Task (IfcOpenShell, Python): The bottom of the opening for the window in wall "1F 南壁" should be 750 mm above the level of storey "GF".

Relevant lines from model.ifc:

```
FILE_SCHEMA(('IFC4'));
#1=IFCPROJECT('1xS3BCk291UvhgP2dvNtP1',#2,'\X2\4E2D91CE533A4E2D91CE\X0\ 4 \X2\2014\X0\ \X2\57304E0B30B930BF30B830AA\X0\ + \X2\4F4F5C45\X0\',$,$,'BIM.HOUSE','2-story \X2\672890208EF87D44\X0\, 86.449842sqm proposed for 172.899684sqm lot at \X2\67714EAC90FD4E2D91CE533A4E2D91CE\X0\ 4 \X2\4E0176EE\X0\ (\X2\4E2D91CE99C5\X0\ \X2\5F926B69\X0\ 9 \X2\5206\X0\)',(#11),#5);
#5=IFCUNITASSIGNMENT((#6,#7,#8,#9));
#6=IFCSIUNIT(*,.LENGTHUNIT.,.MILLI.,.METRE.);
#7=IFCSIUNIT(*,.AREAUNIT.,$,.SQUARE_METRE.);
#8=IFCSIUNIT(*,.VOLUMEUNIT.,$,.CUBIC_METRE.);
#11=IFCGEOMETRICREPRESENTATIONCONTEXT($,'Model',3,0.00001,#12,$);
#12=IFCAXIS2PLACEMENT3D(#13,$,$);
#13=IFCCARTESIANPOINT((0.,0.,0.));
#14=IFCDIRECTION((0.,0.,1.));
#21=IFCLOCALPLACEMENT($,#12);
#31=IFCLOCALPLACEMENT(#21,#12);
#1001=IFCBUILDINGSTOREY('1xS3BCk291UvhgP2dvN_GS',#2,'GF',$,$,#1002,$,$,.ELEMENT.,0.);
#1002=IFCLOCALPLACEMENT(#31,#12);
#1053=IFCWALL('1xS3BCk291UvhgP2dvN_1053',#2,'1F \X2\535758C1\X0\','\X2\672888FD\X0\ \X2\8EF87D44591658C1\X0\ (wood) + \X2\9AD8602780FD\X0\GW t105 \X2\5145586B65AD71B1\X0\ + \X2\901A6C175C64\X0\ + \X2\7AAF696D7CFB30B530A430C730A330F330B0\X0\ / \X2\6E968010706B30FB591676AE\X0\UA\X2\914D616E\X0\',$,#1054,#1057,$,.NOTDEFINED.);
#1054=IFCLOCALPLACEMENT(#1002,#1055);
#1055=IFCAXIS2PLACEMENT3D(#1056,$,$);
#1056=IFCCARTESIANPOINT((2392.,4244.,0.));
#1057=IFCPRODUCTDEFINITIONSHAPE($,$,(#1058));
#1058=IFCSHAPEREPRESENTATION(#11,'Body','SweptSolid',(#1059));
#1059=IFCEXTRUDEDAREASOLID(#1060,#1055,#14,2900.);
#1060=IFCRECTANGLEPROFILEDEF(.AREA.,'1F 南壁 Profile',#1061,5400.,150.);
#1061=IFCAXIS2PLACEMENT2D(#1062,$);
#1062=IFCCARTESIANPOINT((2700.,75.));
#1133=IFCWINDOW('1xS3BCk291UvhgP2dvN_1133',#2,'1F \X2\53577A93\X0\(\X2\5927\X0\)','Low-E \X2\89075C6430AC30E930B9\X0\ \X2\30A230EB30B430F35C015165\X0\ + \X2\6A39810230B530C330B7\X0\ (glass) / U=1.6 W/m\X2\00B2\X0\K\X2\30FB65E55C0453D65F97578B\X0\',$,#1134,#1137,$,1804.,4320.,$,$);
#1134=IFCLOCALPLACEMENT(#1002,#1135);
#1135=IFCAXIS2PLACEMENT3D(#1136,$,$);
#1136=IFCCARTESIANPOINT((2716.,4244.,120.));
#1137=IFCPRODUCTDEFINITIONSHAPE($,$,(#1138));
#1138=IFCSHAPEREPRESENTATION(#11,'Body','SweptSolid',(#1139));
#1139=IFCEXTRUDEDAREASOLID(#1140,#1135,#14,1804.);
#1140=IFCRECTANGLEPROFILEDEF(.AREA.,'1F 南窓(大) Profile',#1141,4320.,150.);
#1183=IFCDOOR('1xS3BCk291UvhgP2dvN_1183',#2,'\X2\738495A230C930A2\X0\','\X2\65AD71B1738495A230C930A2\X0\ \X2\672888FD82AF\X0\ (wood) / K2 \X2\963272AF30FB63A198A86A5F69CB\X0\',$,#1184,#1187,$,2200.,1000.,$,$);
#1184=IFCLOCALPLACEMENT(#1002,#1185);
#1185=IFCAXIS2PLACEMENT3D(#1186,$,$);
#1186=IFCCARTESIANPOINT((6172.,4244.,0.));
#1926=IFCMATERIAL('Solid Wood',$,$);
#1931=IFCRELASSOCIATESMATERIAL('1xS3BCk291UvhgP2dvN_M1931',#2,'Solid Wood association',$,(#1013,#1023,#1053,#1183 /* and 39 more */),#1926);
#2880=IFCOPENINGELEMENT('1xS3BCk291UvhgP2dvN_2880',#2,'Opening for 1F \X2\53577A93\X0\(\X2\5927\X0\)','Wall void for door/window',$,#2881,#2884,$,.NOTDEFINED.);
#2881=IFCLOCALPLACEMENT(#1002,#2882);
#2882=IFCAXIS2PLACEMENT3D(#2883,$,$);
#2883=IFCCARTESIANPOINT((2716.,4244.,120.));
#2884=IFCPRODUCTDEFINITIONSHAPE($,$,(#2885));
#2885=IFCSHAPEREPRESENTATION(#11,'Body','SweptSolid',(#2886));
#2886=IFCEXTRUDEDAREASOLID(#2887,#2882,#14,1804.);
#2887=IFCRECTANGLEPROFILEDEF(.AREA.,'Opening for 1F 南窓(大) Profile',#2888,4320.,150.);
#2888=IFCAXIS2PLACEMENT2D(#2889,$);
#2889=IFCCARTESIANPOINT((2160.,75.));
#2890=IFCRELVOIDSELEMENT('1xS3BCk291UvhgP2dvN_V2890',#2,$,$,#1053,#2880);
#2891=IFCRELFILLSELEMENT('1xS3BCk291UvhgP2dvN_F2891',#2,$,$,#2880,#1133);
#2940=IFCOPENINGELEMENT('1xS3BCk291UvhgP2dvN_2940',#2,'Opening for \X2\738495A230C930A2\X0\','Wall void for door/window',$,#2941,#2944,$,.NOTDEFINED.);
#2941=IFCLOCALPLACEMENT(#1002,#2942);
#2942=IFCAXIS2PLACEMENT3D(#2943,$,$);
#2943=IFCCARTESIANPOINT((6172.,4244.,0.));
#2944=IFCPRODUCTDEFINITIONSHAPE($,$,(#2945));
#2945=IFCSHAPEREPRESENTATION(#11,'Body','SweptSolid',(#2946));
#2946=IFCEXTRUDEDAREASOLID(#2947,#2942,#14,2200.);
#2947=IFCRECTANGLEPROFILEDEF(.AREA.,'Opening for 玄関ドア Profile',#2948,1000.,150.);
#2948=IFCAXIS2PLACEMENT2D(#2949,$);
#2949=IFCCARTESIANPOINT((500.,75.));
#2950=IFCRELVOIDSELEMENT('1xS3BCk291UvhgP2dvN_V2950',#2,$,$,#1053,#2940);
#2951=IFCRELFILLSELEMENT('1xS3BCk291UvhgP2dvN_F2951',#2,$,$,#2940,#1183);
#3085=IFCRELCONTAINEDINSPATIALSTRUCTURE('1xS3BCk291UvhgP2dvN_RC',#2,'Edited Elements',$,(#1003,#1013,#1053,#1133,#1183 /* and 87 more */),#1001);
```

```python
import numpy as np
import ifcopenshell
import ifcopenshell.api.geometry
import ifcopenshell.geom
import ifcopenshell.util.element
import ifcopenshell.util.placement
import ifcopenshell.util.shape
import ifcopenshell.util.unit

model = ifcopenshell.open("model.ifc")
unit_scale = ifcopenshell.util.unit.calculate_unit_scale(model)

window = model.by_id(1133)
opening = window.FillsVoids[0].RelatingOpeningElement
storey = ifcopenshell.util.element.get_container(window, ifc_class="IfcBuildingStorey")
level = ifcopenshell.util.placement.get_local_placement(storey.ObjectPlacement)[2, 3]

# The opening's origin need not be at the sill, so measure its lowest point.
shape = ifcopenshell.geom.create_shape(ifcopenshell.geom.settings(), opening)
bottom = ifcopenshell.util.shape.get_shape_bottom_elevation(shape, shape.geometry) / unit_scale
dz = level + 750.0 - bottom

shift = np.array([0.0, 0.0, dz])
# The window is not placed relative to its opening, so move both.
for product in (opening, window):
    matrix = ifcopenshell.util.placement.get_local_placement(product.ObjectPlacement)
    matrix[:3, 3] += shift
    ifcopenshell.api.geometry.edit_object_placement(model, product=product, matrix=matrix, is_si=False)

print(f"moved by {dz * unit_scale:+.3f} m")

model.write("model_rev.ifc")
```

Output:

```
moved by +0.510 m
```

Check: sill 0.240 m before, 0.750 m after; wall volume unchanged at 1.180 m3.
